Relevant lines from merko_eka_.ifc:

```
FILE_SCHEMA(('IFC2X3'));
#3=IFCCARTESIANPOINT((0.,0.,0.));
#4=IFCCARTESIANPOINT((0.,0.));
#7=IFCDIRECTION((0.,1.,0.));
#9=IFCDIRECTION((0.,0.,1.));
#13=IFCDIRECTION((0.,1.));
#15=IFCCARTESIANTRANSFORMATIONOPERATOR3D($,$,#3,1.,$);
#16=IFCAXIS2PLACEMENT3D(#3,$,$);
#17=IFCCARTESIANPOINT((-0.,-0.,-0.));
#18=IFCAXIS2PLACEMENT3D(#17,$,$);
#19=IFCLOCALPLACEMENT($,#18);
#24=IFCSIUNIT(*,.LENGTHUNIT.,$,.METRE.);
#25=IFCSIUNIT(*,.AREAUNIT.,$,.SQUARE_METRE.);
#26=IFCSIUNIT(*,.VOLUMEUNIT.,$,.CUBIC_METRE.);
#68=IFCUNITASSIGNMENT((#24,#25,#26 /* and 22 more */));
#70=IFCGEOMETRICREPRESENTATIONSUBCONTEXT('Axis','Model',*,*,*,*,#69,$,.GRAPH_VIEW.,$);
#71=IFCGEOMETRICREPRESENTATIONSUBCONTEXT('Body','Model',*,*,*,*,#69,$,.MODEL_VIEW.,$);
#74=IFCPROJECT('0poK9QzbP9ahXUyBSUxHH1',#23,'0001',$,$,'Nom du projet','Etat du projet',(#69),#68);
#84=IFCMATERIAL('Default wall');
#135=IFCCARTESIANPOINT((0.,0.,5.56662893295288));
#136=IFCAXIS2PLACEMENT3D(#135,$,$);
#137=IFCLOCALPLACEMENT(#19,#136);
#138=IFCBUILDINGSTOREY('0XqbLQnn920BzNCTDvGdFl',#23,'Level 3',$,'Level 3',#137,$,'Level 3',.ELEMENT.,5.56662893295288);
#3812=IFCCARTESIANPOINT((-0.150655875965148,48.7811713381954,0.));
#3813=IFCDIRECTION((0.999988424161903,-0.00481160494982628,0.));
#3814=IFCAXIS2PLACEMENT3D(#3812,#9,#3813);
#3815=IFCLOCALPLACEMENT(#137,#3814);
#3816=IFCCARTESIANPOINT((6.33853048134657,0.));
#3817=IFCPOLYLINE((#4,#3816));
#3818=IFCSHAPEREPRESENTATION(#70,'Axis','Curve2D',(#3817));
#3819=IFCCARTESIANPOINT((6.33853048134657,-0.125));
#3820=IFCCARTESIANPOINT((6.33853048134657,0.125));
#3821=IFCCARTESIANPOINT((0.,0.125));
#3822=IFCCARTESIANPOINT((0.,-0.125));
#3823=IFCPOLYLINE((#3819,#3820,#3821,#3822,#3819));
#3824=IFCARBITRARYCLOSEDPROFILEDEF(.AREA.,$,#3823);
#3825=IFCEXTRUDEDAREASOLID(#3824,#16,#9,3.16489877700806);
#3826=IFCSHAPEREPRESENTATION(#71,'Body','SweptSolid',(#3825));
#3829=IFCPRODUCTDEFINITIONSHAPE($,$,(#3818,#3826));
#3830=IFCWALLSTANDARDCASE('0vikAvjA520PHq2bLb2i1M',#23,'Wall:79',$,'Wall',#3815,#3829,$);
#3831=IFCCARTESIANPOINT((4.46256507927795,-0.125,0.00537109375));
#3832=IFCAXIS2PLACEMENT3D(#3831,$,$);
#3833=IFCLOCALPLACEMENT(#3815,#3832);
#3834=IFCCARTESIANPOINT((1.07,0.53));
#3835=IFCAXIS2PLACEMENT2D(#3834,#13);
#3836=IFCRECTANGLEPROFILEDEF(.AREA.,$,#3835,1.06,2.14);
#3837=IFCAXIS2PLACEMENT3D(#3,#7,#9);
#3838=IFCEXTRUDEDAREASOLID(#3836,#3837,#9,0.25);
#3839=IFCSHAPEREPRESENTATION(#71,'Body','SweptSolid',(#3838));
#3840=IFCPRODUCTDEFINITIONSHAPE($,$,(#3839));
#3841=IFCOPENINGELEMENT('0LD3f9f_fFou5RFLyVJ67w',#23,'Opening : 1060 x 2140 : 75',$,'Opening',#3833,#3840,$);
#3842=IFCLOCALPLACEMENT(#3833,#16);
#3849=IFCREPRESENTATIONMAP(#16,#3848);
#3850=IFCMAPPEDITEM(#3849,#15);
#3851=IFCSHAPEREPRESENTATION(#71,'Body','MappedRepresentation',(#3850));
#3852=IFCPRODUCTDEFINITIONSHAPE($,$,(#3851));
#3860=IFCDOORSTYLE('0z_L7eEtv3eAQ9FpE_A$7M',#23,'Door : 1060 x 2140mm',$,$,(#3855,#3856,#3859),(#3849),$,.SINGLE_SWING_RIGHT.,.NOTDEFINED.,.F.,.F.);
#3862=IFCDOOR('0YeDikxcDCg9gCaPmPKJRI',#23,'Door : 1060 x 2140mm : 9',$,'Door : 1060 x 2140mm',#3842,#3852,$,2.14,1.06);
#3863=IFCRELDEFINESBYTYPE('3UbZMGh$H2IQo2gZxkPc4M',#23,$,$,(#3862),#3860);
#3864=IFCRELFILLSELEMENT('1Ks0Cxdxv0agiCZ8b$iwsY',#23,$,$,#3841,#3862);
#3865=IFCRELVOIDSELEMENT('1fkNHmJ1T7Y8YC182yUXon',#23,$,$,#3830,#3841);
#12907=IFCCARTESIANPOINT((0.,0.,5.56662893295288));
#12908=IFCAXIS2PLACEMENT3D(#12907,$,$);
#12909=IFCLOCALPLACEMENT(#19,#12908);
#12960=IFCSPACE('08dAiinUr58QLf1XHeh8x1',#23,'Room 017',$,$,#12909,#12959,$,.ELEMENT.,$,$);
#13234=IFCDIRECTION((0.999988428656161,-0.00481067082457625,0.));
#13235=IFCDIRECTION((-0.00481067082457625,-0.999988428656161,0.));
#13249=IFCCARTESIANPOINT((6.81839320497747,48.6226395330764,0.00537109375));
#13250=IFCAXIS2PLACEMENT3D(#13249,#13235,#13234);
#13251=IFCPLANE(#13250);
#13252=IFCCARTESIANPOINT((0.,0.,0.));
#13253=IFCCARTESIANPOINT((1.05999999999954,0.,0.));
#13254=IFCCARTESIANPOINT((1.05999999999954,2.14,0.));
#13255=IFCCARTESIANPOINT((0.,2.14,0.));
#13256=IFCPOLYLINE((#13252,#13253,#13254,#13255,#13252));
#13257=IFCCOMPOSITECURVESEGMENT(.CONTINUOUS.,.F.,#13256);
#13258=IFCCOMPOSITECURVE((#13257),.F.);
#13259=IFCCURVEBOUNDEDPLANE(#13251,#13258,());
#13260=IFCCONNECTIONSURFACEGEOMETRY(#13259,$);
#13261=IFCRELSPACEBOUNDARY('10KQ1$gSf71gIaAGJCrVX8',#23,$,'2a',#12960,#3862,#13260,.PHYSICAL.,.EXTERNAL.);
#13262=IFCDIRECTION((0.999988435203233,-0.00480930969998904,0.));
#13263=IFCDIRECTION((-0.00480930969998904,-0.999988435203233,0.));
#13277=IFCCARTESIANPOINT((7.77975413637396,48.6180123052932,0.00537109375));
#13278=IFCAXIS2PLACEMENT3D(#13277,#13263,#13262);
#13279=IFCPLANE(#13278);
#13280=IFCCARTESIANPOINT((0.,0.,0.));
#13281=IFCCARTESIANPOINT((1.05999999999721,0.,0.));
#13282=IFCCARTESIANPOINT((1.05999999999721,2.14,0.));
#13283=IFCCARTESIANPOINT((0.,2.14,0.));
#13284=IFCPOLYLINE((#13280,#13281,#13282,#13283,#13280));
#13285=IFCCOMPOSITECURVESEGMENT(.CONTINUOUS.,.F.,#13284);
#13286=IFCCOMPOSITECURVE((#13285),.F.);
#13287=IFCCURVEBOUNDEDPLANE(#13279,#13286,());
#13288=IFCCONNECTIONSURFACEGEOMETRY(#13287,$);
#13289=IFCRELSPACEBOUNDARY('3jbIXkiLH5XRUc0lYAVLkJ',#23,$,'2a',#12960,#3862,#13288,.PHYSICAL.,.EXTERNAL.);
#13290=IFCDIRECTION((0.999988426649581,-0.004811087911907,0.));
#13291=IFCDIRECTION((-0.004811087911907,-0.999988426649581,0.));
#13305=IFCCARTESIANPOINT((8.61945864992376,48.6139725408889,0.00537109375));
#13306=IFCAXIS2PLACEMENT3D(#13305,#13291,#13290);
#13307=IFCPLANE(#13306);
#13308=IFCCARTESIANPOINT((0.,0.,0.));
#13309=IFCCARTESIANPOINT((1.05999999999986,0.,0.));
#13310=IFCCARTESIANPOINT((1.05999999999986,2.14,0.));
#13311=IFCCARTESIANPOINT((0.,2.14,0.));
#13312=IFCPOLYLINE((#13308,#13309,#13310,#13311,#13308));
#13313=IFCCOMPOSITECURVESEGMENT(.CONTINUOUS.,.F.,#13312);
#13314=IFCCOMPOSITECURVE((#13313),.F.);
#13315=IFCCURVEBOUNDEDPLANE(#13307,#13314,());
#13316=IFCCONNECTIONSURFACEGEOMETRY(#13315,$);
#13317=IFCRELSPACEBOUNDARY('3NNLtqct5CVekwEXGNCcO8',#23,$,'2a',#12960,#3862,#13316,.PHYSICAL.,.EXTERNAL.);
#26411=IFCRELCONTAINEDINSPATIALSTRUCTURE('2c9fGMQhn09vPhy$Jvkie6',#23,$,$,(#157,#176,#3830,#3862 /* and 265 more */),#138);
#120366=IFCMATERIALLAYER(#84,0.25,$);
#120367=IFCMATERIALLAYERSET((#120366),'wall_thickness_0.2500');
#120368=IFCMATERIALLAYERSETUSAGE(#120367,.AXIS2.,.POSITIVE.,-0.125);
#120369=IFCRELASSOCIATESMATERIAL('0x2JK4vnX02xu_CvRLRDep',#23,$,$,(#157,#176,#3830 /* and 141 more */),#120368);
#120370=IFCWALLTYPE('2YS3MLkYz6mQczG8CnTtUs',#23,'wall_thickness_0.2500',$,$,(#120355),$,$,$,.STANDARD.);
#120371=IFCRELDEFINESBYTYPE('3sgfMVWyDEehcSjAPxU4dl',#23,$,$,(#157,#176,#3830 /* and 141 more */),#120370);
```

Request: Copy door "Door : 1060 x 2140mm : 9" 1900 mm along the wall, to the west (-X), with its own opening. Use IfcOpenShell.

```python
import numpy as np
import ifcopenshell
import ifcopenshell.api.feature
import ifcopenshell.api.geometry
import ifcopenshell.api.root
import ifcopenshell.geom
import ifcopenshell.util.element
import ifcopenshell.util.placement
import ifcopenshell.util.shape

model = ifcopenshell.open("merko_eka_.ifc")
settings = ifcopenshell.geom.settings()


def volume(element):
    """Net volume in cubic metres, openings subtracted."""
    shape = ifcopenshell.geom.create_shape(settings, element)
    return ifcopenshell.util.shape.get_volume(shape.geometry)


door = model.by_guid("0YeDikxcDCg9gCaPmPKJRI")
opening = door.FillsVoids[0].RelatingOpeningElement
wall = opening.VoidsElements[0].RelatingBuildingElement
before = volume(wall)
shift = ifcopenshell.util.placement.get_local_placement(wall.ObjectPlacement)[:3, 0] * -1.9

# copy_class copies the void relationship, type, container and properties, but no geometry.
new_opening = ifcopenshell.api.root.copy_class(model, product=opening)
new_opening.Representation = ifcopenshell.util.element.copy_deep(
    model, opening.Representation, exclude=["IfcGeometricRepresentationContext", "IfcRepresentationMap"]
)
new_opening.Name = "Opening : 1060 x 2140"
new_door = ifcopenshell.api.root.copy_class(model, product=door)
new_door.Representation = ifcopenshell.util.element.copy_deep(
    model, door.Representation, exclude=["IfcGeometricRepresentationContext", "IfcRepresentationMap"]
)
new_door.Name = "Door : 1060 x 2140mm"
fills = ifcopenshell.api.feature.add_filling(model, opening=new_opening, element=new_door)
fills.OwnerHistory = new_door.OwnerHistory  # required in IFC2X3

for old, new in ((opening, new_opening), (door, new_door)):
    matrix = ifcopenshell.util.placement.get_local_placement(old.ObjectPlacement)
    matrix[:3, 3] += shift
    ifcopenshell.api.geometry.edit_object_placement(model, product=new, matrix=matrix, is_si=False)

# The copied space boundaries still share their surfaces with the original.
for rel in new_door.ProvidesBoundaries:
    if rel.ConnectionGeometry:
        rel.ConnectionGeometry = ifcopenshell.util.element.copy_deep(model, rel.ConnectionGeometry)

# Space boundary surfaces are stored in each space's coordinates; move them too.
for rel in new_door.ProvidesBoundaries:
    if not rel.ConnectionGeometry:
        continue
    surface = rel.ConnectionGeometry.SurfaceOnRelatingElement.BasisSurface
    space_matrix = ifcopenshell.util.placement.get_local_placement(rel.RelatingSpace.ObjectPlacement)
    point = np.array(surface.Position.Location.Coordinates) + space_matrix[:3, :3].T @ shift
    surface.Position = model.createIfcAxis2Placement3D(
        model.createIfcCartesianPoint(point.tolist()), surface.Position.Axis, surface.Position.RefDirection
    )

after = volume(wall)

print(f"wall volume {before:.3f} -> {after:.3f} m3")

model.write("merko_eka__edited.ifc")
```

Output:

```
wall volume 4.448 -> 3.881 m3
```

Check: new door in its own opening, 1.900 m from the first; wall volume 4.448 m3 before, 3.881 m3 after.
